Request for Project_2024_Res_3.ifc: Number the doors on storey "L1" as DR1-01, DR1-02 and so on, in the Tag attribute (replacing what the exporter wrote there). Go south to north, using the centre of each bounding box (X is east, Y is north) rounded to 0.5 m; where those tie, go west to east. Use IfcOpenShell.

First a look at what the model holds.

```python
import ifcopenshell
import ifcopenshell.util.element
import ifcopenshell.util.placement

model = ifcopenshell.open("Project_2024_Res_3.ifc")
print(model.schema)
storey = next(s for s in model.by_type("IfcBuildingStorey") if s.Name == "L1")
doors = [e for e in ifcopenshell.util.element.get_decomposition(storey) if e.is_a("IfcDoor")]
for e in sorted(doors, key=lambda e: e.id()):
    origin = ifcopenshell.util.placement.get_local_placement(e.ObjectPlacement)[:3, 3]
    print(e.id(), e.Tag, e.Name, origin.round(2) + 0.0, sep=" | ")
```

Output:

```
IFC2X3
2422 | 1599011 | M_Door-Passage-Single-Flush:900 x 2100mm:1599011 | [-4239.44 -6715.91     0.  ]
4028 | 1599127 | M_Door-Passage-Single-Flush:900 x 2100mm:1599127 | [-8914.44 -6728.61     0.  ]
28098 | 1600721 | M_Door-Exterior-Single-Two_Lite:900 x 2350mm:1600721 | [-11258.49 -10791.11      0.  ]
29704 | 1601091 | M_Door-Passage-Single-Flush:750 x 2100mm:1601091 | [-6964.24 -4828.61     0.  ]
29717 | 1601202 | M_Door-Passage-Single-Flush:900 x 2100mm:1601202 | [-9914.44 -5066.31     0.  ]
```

```python
import ifcopenshell
import ifcopenshell.geom
import ifcopenshell.util.element
import ifcopenshell.util.shape

model = ifcopenshell.open("Project_2024_Res_3.ifc")
settings = ifcopenshell.geom.settings()
settings.set("use-world-coords", True)


def centre(element):
    shape = ifcopenshell.geom.create_shape(settings, element)
    return ifcopenshell.util.shape.get_bbox_centroid(shape.geometry)


storey = next(s for s in model.by_type("IfcBuildingStorey") if s.Name == "L1")
doors = [e for e in ifcopenshell.util.element.get_decomposition(storey) if e.is_a("IfcDoor")]

# Insertion points can sit at a corner or the storey origin, so sort by the geometry (in metres).
centres = {e: centre(e) for e in doors}
doors.sort(key=lambda e: (round(centres[e][1] / 0.5), centres[e][0]))

for i, e in enumerate(doors, start=1):
    number = f"DR1-{i:02d}"
    e.Tag = number
    print(e.id(), number)

model.write("Project_2024_Res_3-out.ifc")
```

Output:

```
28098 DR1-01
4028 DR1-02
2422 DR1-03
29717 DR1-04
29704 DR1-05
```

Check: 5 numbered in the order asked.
